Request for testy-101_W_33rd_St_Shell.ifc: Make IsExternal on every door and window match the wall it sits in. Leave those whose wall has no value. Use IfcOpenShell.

First a look at what the model holds.

```python
import ifcopenshell
import ifcopenshell.util.element

model = ifcopenshell.open("testy-101_W_33rd_St_Shell.ifc")
print(model.schema)
seen = {}
for e in model.by_type("IfcDoor") + model.by_type("IfcWindow"):
    if not e.FillsVoids:
        continue
    host = e.FillsVoids[0].RelatingOpeningElement.VoidsElements[0].RelatingBuildingElement
    own = ifcopenshell.util.element.get_pset(e, f"Pset_{e.is_a()[3:].removesuffix('StandardCase')}Common", "IsExternal")
    wall = ifcopenshell.util.element.get_pset(host, "Pset_WallCommon", "IsExternal")
    seen[e.is_a(), own, wall] = seen.get((e.is_a(), own, wall), 0) + 1
for (cls, own, wall), count in sorted(seen.items(), key=str):
    print(count, cls, "IsExternal:", own, "| host wall:", wall)
```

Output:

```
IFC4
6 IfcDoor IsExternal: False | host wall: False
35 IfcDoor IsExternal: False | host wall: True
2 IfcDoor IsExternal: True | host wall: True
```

```python
import ifcopenshell
import ifcopenshell.api.pset
import ifcopenshell.util.element

model = ifcopenshell.open("testy-101_W_33rd_St_Shell.ifc")

count = 0
for ifc_class, pset_name in (("IfcDoor", "Pset_DoorCommon"), ("IfcWindow", "Pset_WindowCommon")):
    for e in model.by_type(ifc_class):
        if not e.FillsVoids:
            continue
        host = e.FillsVoids[0].RelatingOpeningElement.VoidsElements[0].RelatingBuildingElement
        external = ifcopenshell.util.element.get_pset(host, "Pset_WallCommon", "IsExternal")
        if external is None or ifcopenshell.util.element.get_pset(e, pset_name, "IsExternal") == external:
            continue
        pset = ifcopenshell.api.pset.add_pset(model, product=e, name=pset_name)
        ifcopenshell.api.pset.edit_pset(model, pset=pset, properties={"IsExternal": external})
        count += 1

print(count, "updated")

model.write("testy-101_W_33rd_St_Shell_edited.ifc")
```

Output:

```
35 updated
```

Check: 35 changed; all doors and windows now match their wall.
